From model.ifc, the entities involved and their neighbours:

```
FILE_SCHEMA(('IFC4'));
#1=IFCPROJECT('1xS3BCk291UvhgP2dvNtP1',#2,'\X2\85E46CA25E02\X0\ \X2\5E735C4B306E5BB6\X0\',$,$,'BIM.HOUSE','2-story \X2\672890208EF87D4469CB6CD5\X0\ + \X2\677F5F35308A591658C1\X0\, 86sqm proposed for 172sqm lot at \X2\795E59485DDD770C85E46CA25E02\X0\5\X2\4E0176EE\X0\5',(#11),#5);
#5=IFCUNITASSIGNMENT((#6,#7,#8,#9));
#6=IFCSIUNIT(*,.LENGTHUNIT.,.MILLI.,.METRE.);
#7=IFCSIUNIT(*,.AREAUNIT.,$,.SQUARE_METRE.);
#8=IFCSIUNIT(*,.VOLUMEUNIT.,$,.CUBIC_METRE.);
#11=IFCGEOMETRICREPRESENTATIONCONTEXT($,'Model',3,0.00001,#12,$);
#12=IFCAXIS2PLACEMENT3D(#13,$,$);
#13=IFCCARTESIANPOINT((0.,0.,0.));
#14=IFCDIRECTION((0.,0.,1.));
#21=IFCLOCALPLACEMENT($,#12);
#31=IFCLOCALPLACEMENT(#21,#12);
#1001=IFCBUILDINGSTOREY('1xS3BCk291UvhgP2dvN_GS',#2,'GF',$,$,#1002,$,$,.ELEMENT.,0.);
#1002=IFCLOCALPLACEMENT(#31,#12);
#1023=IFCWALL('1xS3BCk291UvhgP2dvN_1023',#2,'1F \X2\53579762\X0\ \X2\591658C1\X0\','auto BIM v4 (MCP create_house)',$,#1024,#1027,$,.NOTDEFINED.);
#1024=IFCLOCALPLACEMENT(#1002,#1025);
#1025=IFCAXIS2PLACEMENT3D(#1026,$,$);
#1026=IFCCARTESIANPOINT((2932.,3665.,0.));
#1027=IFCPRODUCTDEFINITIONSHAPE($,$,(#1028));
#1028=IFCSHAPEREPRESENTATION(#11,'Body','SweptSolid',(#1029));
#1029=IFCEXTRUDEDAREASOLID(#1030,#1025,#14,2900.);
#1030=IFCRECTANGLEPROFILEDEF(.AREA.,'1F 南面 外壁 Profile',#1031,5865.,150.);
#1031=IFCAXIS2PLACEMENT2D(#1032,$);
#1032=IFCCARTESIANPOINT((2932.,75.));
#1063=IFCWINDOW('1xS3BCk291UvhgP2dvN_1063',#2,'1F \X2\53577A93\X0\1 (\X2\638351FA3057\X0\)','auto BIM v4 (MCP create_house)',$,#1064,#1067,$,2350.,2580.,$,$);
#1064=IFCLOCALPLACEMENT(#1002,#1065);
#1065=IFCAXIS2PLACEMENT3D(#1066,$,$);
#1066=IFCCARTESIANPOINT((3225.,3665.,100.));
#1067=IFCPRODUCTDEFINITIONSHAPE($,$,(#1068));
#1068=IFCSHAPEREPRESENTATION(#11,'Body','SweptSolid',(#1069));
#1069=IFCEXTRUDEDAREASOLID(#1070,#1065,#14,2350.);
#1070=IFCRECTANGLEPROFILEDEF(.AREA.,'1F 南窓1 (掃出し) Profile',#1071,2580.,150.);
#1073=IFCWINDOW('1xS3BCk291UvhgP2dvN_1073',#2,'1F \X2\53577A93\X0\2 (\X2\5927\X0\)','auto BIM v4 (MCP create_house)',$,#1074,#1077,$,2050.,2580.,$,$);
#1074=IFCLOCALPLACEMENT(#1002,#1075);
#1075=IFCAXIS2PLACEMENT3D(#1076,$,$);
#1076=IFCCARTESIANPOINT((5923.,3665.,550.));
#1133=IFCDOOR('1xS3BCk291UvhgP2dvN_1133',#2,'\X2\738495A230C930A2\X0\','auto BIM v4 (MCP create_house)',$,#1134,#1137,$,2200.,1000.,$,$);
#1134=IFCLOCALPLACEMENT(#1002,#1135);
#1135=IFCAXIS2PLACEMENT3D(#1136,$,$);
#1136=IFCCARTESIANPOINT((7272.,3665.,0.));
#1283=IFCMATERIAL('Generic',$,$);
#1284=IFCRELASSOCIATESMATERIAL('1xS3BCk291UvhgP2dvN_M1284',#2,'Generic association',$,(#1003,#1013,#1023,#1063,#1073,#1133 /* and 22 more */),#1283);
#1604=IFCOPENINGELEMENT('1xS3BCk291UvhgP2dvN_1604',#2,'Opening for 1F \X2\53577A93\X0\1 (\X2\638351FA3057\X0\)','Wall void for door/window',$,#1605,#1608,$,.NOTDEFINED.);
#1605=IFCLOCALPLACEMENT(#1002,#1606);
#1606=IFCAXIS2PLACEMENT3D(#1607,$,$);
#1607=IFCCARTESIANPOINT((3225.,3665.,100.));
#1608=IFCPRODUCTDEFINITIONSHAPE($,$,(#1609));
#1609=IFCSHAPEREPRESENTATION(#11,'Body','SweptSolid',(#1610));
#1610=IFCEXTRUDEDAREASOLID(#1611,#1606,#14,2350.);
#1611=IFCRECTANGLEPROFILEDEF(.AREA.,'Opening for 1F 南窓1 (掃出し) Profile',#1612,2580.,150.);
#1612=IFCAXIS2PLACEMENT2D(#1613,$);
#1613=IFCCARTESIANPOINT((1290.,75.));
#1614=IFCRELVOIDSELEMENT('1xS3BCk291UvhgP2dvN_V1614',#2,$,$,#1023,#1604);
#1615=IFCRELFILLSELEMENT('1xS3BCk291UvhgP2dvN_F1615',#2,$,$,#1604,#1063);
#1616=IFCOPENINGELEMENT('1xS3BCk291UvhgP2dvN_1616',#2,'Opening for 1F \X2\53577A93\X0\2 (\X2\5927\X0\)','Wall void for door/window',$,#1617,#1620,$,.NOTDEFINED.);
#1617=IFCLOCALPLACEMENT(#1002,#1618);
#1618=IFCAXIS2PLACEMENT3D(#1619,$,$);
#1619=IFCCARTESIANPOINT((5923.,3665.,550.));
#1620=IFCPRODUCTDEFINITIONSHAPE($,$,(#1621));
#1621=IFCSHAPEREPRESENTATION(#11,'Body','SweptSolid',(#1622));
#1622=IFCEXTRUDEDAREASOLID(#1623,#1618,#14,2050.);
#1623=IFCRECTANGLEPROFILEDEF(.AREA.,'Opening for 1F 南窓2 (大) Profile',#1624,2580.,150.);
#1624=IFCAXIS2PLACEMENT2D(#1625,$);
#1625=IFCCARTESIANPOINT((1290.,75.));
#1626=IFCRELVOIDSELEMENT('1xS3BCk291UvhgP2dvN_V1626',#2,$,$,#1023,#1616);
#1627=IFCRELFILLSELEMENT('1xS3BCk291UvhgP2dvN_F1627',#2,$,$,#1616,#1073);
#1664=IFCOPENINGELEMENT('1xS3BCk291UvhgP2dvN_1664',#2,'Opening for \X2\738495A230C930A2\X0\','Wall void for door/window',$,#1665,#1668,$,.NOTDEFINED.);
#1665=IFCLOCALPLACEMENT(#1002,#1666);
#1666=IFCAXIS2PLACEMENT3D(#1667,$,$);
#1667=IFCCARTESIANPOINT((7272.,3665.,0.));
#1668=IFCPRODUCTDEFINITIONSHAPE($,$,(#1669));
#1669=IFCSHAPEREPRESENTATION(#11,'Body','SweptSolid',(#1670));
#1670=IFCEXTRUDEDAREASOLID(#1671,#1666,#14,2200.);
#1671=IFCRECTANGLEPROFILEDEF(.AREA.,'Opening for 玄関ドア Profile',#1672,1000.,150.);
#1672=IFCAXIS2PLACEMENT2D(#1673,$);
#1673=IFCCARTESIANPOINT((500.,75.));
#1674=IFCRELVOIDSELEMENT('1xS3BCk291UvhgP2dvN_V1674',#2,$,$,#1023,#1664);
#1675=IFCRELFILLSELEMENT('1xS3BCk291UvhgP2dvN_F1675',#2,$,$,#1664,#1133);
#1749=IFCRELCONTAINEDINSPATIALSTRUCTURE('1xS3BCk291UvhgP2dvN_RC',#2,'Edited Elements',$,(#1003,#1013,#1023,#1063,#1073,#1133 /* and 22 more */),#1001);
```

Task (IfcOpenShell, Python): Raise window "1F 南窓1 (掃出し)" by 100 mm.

```python
import numpy as np
import ifcopenshell
import ifcopenshell.api.geometry
import ifcopenshell.util.placement
import ifcopenshell.util.unit

model = ifcopenshell.open("model.ifc")
unit_scale = ifcopenshell.util.unit.calculate_unit_scale(model)

window = model.by_guid("1xS3BCk291UvhgP2dvN_1063")
opening = window.FillsVoids[0].RelatingOpeningElement
dz = 100.0

shift = np.array([0.0, 0.0, dz])
# The window is not placed relative to its opening, so move both.
for product in (opening, window):
    matrix = ifcopenshell.util.placement.get_local_placement(product.ObjectPlacement)
    matrix[:3, 3] += shift
    ifcopenshell.api.geometry.edit_object_placement(model, product=product, matrix=matrix, is_si=False)

print(f"moved by {dz * unit_scale:+.3f} m")

model.write("model_updated.ifc")
```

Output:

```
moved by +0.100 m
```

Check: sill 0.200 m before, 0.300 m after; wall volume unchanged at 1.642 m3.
